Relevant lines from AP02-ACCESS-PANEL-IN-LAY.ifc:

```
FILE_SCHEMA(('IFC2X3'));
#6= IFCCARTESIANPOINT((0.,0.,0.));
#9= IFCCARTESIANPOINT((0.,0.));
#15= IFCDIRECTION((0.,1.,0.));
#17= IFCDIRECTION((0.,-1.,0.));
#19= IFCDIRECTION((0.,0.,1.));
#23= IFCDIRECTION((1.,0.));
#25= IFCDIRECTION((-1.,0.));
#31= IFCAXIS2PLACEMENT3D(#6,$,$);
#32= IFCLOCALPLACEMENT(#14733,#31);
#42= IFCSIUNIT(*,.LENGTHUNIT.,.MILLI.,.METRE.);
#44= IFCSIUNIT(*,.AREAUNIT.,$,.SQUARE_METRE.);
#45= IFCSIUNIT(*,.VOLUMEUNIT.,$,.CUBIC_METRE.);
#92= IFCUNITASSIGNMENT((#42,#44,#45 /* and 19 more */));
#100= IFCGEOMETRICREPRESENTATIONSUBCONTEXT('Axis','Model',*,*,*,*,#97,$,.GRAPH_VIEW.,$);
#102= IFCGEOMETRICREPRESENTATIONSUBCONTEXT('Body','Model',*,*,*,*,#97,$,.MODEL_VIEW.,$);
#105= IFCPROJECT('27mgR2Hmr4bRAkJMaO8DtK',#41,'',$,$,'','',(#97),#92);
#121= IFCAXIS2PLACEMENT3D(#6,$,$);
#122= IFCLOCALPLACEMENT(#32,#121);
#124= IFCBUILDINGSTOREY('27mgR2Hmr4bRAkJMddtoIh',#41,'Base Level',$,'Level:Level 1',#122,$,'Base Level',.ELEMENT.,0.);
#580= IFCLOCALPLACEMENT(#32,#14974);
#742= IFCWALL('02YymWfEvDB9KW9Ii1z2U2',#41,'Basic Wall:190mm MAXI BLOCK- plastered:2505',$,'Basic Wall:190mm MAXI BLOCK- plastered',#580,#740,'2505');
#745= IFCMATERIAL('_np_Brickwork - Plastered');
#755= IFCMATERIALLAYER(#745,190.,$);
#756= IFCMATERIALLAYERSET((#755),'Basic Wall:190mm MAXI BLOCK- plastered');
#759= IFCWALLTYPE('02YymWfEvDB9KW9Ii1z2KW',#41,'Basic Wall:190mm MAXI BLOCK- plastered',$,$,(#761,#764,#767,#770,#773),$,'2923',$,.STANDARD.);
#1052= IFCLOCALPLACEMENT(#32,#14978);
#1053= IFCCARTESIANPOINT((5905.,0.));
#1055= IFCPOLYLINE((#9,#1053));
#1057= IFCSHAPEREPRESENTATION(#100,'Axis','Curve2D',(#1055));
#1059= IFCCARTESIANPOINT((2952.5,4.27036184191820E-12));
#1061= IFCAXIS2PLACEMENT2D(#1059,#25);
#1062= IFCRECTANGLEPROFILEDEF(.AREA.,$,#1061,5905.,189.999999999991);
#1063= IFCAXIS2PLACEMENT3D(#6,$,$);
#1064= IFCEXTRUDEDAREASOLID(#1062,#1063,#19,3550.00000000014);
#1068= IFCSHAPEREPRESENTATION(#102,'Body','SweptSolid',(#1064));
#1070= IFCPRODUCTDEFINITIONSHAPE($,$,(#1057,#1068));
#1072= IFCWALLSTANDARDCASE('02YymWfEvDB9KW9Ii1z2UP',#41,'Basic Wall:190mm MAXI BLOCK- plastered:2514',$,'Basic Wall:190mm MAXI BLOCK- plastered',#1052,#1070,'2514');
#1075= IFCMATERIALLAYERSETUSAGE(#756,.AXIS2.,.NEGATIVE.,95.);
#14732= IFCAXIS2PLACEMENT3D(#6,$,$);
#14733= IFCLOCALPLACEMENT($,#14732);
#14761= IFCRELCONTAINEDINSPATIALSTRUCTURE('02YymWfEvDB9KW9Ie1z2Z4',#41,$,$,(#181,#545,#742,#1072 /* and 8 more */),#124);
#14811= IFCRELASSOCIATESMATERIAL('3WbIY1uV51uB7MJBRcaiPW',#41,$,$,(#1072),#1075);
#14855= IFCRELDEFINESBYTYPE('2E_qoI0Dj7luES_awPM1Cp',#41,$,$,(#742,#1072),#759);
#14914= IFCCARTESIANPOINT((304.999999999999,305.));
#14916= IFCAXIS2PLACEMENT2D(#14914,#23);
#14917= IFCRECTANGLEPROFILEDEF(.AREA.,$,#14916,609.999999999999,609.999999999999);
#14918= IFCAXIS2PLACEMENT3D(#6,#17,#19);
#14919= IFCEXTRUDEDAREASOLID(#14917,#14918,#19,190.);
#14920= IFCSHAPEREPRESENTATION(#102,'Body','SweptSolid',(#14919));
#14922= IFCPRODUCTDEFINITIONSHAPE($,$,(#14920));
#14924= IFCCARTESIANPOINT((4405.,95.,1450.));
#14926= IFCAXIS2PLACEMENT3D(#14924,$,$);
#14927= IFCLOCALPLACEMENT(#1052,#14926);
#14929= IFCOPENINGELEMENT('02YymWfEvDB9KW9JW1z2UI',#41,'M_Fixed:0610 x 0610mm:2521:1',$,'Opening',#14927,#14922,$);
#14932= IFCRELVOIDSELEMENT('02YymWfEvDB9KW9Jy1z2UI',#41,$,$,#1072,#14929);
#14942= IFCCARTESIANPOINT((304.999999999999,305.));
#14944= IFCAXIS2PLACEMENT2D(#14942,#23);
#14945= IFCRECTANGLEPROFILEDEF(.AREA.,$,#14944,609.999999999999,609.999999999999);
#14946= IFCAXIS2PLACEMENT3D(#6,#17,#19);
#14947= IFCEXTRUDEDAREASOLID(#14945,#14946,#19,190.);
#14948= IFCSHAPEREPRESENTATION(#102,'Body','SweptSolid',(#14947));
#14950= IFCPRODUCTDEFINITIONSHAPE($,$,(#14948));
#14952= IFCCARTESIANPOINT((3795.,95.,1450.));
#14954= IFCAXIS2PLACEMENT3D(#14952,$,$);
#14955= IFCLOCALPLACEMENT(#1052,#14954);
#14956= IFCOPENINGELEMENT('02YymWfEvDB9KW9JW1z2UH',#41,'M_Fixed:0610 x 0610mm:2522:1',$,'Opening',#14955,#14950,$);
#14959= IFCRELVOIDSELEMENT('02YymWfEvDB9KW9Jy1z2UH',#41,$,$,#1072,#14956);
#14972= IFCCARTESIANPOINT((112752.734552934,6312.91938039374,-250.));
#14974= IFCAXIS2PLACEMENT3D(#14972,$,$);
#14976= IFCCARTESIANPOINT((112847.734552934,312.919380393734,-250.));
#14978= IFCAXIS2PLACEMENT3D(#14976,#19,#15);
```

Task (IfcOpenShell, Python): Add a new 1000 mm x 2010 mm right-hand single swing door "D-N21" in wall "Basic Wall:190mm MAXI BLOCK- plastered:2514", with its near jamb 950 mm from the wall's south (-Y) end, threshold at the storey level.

```python
import numpy as np
import ifcopenshell
import ifcopenshell.api.feature
import ifcopenshell.api.geometry
import ifcopenshell.api.root
import ifcopenshell.api.spatial
import ifcopenshell.api.type
import ifcopenshell.geom
import ifcopenshell.util.element
import ifcopenshell.util.placement
import ifcopenshell.util.representation
import ifcopenshell.util.shape
import ifcopenshell.util.unit

model = ifcopenshell.open("AP02-ACCESS-PANEL-IN-LAY.ifc")
unit_scale = ifcopenshell.util.unit.calculate_unit_scale(model)
settings = ifcopenshell.geom.settings()


def volume(element):
    """Net volume in cubic metres, openings subtracted."""
    shape = ifcopenshell.geom.create_shape(settings, element)
    return ifcopenshell.util.shape.get_volume(shape.geometry)


wall = model.by_guid("02YymWfEvDB9KW9Ii1z2UP")
storey = ifcopenshell.util.element.get_container(wall, ifc_class="IfcBuildingStorey")
context = ifcopenshell.util.representation.get_context(model, "Model", "Body", "MODEL_VIEW")
before = volume(wall)

width, height, from_end, sill = 1, 2.01, 0.95, 0.0  # metres

# The wall runs along its own X axis, and the end named is its -X end.
wall_shape = ifcopenshell.geom.create_shape(settings, wall)
x, y, z = ifcopenshell.util.shape.get_vertices(wall_shape.geometry).T
start = x.min() + from_end
face, thickness = float(y.min()), float(y.max() - y.min())
wall_matrix = ifcopenshell.util.placement.get_local_placement(wall.ObjectPlacement)
level = ifcopenshell.util.placement.get_local_placement(storey.ObjectPlacement)[2, 3]


def in_wall(x, y):
    """Placement at x, y metres in the wall's axes, at sill height."""
    matrix = wall_matrix.copy()
    matrix[:, 3] = wall_matrix @ np.array([x / unit_scale, y / unit_scale, 0.0, 1.0])
    matrix[2, 3] = level + sill / unit_scale
    return matrix


# Opening: a box that overshoots both wall faces by 50 mm.
opening = ifcopenshell.api.root.create_entity(model, ifc_class="IfcOpeningElement")
box = ifcopenshell.api.geometry.add_wall_representation(
    model, context=context, length=width, height=height, thickness=thickness + 0.1
)
ifcopenshell.api.geometry.assign_representation(model, product=opening, representation=box)
ifcopenshell.api.geometry.edit_object_placement(model, product=opening, matrix=in_wall(start, face - 0.05), is_si=False)
ifcopenshell.api.feature.add_feature(model, feature=opening, element=wall)

door = ifcopenshell.api.root.create_entity(model, ifc_class="IfcDoor", name="D-N21")
door.OverallWidth, door.OverallHeight = width / unit_scale, height / unit_scale
body = ifcopenshell.api.geometry.add_door_representation(
    model,
    context=context,
    overall_width=door.OverallWidth,
    overall_height=door.OverallHeight,
    operation_type="SINGLE_SWING_RIGHT",
    lining_properties={"LiningDepth": thickness / unit_scale, "ThresholdDepth": thickness / unit_scale},
)
ifcopenshell.api.geometry.assign_representation(model, product=door, representation=body)
ifcopenshell.api.spatial.assign_container(model, products=[door], relating_structure=storey)
fills = ifcopenshell.api.feature.add_filling(model, opening=opening, element=door)
fills.OwnerHistory = door.OwnerHistory  # required in IFC2X3

# IFC2X3 keeps the operation on the door style.
style = ifcopenshell.api.root.create_entity(model, ifc_class="IfcDoorStyle", name="D-N21")
style.OperationType, style.ConstructionType = "SINGLE_SWING_RIGHT", "NOTDEFINED"
style.ParameterTakesPrecedence = style.Sizeable = False
ifcopenshell.api.type.assign_type(model, related_objects=[door], relating_type=style)

# The lining spans the wall, so the door starts at the wall face.
ifcopenshell.api.geometry.edit_object_placement(model, product=door, matrix=in_wall(start, face), is_si=False)

after = volume(wall)

print(f"wall volume {before:.3f} -> {after:.3f} m3")

model.write("AP02-ACCESS-PANEL-IN-LAY_rev.ifc")
```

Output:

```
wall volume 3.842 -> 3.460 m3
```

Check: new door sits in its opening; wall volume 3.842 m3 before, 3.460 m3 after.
